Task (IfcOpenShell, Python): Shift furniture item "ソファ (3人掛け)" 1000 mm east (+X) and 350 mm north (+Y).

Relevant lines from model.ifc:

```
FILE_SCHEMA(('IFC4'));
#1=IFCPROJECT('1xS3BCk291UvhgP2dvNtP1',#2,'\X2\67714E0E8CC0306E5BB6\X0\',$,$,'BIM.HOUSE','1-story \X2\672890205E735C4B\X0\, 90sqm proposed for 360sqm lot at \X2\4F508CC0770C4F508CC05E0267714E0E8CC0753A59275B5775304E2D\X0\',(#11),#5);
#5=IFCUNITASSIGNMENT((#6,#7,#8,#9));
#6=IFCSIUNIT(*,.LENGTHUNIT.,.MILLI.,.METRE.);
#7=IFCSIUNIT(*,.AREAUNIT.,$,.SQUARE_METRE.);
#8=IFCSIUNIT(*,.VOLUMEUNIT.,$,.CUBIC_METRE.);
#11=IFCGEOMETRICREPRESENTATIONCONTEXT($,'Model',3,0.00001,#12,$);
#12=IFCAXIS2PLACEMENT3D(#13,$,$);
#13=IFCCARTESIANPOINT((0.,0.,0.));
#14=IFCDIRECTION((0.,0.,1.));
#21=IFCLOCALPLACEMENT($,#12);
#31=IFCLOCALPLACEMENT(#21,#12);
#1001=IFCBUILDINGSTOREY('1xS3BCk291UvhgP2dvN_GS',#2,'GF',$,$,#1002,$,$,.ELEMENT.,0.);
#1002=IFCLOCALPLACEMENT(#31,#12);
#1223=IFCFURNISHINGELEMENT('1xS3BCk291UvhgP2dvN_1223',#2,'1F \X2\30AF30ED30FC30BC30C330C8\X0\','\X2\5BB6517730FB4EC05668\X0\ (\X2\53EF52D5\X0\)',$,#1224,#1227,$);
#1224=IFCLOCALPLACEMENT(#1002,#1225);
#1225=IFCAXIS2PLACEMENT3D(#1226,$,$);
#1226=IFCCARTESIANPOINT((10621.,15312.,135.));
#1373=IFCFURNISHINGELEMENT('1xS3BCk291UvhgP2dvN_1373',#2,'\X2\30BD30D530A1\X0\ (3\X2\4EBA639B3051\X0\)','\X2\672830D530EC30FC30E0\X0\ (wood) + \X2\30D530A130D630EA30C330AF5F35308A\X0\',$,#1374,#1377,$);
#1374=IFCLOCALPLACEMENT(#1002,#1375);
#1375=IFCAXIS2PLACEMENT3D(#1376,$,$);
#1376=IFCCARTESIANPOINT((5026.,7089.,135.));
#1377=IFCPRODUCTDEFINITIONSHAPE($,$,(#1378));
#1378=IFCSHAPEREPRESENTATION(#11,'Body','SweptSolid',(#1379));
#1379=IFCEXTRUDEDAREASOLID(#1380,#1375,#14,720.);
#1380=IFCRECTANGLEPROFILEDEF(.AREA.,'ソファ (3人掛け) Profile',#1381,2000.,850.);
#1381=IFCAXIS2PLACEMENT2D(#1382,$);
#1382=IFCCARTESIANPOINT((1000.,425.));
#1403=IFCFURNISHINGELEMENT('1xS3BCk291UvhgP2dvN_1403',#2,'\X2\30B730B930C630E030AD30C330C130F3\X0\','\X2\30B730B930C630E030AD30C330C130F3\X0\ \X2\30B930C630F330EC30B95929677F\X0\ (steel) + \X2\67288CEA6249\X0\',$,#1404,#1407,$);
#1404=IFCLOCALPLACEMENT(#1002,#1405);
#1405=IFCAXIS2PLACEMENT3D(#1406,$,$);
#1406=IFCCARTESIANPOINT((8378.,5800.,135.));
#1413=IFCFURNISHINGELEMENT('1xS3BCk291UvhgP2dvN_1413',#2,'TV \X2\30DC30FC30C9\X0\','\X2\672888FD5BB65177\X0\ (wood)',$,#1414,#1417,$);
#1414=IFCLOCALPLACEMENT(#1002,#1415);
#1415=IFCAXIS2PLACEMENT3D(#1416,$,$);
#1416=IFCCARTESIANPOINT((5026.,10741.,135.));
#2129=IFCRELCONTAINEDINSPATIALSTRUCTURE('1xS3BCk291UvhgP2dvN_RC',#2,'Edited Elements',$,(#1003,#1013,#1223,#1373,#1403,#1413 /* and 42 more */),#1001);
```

```python
import ifcopenshell
import ifcopenshell.api.geometry
import ifcopenshell.util.placement
import ifcopenshell.util.unit

model = ifcopenshell.open("model.ifc")
unit_scale = ifcopenshell.util.unit.calculate_unit_scale(model)

item = model.by_id(1373)
matrix = ifcopenshell.util.placement.get_local_placement(item.ObjectPlacement)
matrix[0, 3] += 1 / unit_scale
matrix[1, 3] += 0.35 / unit_scale
ifcopenshell.api.geometry.edit_object_placement(model, product=item, matrix=matrix, is_si=False)

print(ifcopenshell.util.placement.get_local_placement(item.ObjectPlacement).round(3) + 0.0)

model.write("model_rev.ifc")
```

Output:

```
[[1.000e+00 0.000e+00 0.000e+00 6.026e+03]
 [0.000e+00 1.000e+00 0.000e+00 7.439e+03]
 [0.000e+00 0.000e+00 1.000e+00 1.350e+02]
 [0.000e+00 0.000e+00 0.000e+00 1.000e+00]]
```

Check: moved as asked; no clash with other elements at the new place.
